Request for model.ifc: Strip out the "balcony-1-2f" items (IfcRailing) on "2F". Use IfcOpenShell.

First a look at what the model holds.

```python
import ifcopenshell
import ifcopenshell.util.element

model = ifcopenshell.open("model.ifc")
print(model.schema)
storey = next(s for s in model.by_type("IfcBuildingStorey") if s.Name == "2F")
railings = [e for e in ifcopenshell.util.element.get_decomposition(storey) if e.is_a("IfcRailing")]
seen = {}
for e in railings:
    element_type = ifcopenshell.util.element.get_type(e)
    name = element_type.Name if element_type not in (None, e) else None
    seen[name] = seen.get(name, 0) + 1
for name, count in sorted(seen.items(), key=str):
    print(count, "x", name)
```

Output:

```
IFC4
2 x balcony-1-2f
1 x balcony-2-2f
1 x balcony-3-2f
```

```python
import ifcopenshell
import ifcopenshell.api.root
import ifcopenshell.util.element

model = ifcopenshell.open("model.ifc")

storey = next(s for s in model.by_type("IfcBuildingStorey") if s.Name == "2F")
railings = [e for e in ifcopenshell.util.element.get_decomposition(storey) if e.is_a("IfcRailing")]
targets = [e for e in railings if (t := ifcopenshell.util.element.get_type(e)) not in (None, e) and t.Name == "balcony-1-2f"]

for e in targets:
    ifcopenshell.api.root.remove_product(model, product=e)
print(len(targets), "removed")

model.write("model-out.ifc")
```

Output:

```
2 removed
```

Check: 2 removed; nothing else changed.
